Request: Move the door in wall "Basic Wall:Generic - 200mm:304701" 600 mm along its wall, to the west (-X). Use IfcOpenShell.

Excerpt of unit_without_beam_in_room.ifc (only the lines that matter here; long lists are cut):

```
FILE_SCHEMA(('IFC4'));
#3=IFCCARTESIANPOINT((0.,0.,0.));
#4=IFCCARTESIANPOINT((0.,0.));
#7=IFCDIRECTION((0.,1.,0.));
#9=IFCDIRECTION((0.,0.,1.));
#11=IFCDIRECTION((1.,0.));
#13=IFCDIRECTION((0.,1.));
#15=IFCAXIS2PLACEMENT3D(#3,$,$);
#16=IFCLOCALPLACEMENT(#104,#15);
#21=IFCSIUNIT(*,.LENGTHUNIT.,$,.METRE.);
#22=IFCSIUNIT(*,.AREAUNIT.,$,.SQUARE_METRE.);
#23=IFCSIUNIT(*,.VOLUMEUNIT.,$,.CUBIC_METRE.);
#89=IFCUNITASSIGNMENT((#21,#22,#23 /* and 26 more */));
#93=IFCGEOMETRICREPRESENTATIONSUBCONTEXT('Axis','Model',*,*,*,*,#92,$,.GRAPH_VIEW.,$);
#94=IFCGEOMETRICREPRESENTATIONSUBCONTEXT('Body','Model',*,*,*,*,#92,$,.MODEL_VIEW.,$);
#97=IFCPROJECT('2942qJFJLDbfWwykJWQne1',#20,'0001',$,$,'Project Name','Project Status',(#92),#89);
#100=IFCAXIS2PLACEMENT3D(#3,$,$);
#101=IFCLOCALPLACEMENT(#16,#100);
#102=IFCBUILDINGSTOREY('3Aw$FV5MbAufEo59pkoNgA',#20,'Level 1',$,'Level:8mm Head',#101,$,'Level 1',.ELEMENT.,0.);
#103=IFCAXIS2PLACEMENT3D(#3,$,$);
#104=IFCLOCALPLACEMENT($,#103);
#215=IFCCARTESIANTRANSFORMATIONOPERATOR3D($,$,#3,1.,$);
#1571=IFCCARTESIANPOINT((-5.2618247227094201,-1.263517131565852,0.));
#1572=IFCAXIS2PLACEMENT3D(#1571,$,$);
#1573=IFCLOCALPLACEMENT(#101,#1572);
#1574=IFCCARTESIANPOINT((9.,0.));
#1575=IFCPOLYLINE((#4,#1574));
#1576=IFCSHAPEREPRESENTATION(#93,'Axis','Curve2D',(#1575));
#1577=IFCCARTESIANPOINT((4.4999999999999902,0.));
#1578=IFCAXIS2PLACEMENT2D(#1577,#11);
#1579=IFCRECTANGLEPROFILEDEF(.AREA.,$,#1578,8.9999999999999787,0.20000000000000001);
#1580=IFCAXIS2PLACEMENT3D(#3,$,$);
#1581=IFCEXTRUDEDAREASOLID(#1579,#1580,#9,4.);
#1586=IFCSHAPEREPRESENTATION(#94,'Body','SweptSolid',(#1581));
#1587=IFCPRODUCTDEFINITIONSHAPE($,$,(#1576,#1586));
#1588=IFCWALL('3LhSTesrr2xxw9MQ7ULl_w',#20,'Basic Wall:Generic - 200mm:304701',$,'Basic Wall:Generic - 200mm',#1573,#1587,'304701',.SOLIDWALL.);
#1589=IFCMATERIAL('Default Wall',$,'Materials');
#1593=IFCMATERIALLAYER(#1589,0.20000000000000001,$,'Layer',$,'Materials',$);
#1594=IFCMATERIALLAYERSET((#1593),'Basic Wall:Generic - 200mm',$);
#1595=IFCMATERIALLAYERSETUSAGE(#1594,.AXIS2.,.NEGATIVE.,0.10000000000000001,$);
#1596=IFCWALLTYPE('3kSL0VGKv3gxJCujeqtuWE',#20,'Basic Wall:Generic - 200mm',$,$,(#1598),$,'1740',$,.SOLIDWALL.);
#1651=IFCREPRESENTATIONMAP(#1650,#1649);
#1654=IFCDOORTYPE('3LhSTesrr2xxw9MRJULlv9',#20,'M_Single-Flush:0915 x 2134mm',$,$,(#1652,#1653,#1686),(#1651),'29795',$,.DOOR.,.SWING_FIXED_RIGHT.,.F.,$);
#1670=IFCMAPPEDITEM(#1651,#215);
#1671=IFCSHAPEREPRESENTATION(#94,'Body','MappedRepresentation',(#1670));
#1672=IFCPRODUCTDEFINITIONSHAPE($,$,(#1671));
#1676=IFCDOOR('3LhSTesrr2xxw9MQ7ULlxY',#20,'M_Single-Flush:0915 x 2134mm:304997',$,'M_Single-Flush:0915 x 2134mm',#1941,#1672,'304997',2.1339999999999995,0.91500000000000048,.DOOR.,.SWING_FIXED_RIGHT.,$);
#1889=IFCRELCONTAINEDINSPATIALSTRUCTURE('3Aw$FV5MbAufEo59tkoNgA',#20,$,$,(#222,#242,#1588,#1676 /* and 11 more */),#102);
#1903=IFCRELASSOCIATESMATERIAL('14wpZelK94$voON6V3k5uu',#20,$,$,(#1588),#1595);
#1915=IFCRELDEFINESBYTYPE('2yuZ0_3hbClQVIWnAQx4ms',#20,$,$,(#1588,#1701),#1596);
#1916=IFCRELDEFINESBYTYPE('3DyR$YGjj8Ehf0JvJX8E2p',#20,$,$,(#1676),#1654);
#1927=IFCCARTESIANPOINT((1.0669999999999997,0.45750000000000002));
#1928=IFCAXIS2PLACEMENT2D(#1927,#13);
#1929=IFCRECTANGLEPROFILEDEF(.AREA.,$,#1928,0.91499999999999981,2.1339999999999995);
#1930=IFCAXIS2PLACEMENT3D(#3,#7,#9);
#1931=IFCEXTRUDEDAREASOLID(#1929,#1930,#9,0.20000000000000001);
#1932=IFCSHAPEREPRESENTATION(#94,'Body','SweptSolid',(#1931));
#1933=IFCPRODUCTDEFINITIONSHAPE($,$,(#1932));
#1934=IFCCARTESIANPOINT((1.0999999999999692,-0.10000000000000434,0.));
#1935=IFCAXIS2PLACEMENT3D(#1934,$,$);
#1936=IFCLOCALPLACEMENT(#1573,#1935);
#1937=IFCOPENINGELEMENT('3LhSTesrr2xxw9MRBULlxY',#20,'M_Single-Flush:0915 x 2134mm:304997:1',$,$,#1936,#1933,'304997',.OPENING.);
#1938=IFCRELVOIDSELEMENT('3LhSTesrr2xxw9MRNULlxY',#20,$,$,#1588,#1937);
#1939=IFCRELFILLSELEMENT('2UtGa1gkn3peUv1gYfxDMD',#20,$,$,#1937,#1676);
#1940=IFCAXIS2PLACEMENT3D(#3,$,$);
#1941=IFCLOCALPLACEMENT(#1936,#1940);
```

```python
import ifcopenshell
import ifcopenshell.api.geometry
import ifcopenshell.util.placement
import ifcopenshell.util.unit

model = ifcopenshell.open("unit_without_beam_in_room.ifc")
unit_scale = ifcopenshell.util.unit.calculate_unit_scale(model)

door = model.by_id(1676)
opening = door.FillsVoids[0].RelatingOpeningElement
wall = opening.VoidsElements[0].RelatingBuildingElement

wall_matrix = ifcopenshell.util.placement.get_local_placement(wall.ObjectPlacement)
shift = wall_matrix[:3, 0] * -0.6 / unit_scale
before = ifcopenshell.util.placement.get_local_placement(door.ObjectPlacement)[:3, 3].copy()

# The door is placed relative to its opening, so it follows when the opening moves.
matrix = ifcopenshell.util.placement.get_local_placement(opening.ObjectPlacement)
matrix[:3, 3] += shift
ifcopenshell.api.geometry.edit_object_placement(
    model, product=opening, matrix=matrix, is_si=False, should_transform_children=True
)

after = ifcopenshell.util.placement.get_local_placement(door.ObjectPlacement)[:3, 3]
print("door moved by", (after - before).round(3) + 0.0)

model.write("unit_without_beam_in_room_edited.ifc")
```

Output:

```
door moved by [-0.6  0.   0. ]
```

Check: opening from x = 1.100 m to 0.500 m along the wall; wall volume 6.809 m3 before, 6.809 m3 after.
